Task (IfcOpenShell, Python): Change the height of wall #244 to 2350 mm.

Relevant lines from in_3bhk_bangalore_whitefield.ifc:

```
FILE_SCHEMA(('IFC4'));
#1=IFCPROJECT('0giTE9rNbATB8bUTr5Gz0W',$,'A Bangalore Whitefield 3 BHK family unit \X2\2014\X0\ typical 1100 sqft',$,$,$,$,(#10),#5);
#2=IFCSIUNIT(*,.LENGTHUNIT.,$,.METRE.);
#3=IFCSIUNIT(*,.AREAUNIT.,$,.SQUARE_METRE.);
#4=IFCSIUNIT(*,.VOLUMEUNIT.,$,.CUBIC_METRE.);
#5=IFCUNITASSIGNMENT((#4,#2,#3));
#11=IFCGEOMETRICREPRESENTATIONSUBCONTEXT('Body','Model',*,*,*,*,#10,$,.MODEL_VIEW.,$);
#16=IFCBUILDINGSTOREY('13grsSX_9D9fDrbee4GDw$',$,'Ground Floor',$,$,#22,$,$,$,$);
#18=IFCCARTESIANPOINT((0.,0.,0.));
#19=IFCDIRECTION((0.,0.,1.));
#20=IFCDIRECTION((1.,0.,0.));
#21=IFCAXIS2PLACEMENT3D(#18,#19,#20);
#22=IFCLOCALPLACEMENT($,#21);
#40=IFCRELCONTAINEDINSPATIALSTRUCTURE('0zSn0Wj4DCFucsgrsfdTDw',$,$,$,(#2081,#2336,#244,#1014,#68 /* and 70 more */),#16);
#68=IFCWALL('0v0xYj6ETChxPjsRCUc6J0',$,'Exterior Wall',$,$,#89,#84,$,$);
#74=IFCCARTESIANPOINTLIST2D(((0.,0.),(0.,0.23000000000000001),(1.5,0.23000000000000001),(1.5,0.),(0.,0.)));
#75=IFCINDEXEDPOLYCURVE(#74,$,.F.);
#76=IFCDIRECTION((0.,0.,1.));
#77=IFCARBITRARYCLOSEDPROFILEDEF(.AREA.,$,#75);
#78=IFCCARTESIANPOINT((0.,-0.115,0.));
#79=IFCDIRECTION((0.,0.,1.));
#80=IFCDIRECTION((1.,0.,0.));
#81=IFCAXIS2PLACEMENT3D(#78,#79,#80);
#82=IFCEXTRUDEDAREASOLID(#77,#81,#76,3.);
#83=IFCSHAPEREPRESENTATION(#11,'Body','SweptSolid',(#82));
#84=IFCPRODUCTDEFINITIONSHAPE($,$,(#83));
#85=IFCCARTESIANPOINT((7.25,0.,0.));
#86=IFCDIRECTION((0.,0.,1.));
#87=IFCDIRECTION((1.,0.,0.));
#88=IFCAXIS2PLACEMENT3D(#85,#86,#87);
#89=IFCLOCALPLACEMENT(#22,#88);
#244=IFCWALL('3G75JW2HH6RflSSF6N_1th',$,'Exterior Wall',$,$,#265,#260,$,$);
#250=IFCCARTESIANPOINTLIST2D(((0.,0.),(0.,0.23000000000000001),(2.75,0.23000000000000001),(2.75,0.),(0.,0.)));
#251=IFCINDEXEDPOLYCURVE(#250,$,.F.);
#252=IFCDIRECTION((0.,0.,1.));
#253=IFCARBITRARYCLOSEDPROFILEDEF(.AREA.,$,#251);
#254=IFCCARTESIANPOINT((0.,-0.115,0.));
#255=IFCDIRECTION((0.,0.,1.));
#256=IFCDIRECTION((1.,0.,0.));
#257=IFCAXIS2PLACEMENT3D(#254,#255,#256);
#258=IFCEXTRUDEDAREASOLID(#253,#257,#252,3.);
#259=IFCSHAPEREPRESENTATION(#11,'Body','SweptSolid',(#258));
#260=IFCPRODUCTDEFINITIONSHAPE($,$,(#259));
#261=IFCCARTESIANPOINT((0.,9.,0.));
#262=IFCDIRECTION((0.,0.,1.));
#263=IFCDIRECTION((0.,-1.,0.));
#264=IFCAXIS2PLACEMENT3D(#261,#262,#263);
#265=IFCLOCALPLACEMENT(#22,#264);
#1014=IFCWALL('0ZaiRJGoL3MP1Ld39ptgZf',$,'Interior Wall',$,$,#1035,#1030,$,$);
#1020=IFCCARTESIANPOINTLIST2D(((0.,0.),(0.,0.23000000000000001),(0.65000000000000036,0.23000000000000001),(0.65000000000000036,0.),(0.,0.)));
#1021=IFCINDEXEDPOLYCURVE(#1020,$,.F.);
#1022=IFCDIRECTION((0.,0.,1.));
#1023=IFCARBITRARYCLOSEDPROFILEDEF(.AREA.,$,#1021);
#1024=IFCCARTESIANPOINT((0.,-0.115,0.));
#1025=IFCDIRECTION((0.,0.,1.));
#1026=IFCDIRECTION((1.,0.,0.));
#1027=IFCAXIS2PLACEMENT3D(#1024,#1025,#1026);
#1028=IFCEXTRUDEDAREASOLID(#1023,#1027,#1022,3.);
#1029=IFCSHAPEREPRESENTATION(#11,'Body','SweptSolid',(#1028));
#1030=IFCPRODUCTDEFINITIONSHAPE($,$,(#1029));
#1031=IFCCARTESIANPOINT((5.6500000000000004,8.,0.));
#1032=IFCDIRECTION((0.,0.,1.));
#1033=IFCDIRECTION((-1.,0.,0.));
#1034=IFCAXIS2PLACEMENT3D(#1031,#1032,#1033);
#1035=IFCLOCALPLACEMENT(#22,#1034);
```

```python
import ifcopenshell
import ifcopenshell.geom
import ifcopenshell.util.representation
import ifcopenshell.util.shape
import ifcopenshell.util.unit

model = ifcopenshell.open("in_3bhk_bangalore_whitefield.ifc")
unit_scale = ifcopenshell.util.unit.calculate_unit_scale(model)
settings = ifcopenshell.geom.settings()


def volume(element):
    """Net volume in cubic metres, openings subtracted."""
    shape = ifcopenshell.geom.create_shape(settings, element)
    return ifcopenshell.util.shape.get_volume(shape.geometry)


wall = model.by_id(244)
before = volume(wall)

body = ifcopenshell.util.representation.get_representation(wall, "Model", "Body")
solid = body.Items[0]
old_height = solid.Depth
solid.Depth = 2.35 / unit_scale
after = volume(wall)

print(f"height {old_height:g} -> {solid.Depth:g}, volume {before:.3f} -> {after:.3f} m3")

model.write("in_3bhk_bangalore_whitefield_updated.ifc")
```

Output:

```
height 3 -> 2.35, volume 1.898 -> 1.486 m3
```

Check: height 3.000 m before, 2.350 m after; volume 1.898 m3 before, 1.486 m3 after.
